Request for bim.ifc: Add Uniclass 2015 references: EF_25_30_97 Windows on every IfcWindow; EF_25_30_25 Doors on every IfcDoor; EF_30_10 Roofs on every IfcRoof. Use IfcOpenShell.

First a look at what the model holds.

```python
import ifcopenshell

model = ifcopenshell.open("bim.ifc")
print(model.schema)
print("classifications:", [c.Name for c in model.by_type("IfcClassification")])
for ifc_class in ("IfcDoor", "IfcRoof", "IfcStair", "IfcWall", "IfcWindow"):
    print(ifc_class, len(model.by_type(ifc_class)))
```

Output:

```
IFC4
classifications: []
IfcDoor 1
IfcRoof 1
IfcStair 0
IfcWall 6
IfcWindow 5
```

```python
import ifcopenshell
import ifcopenshell.api.classification

model = ifcopenshell.open("bim.ifc")

system = ifcopenshell.api.classification.add_classification(model, classification="Uniclass 2015")

codes = {
    "IfcWindow": ("EF_25_30_97", "Windows"),
    "IfcDoor": ("EF_25_30_25", "Doors"),
    "IfcRoof": ("EF_30_10", "Roofs"),
}
for ifc_class, (code, name) in codes.items():
    products = model.by_type(ifc_class)
    ifcopenshell.api.classification.add_reference(
        model, products=products, classification=system, identification=code, name=name
    )
    print(code, len(products))

model.write("bim_v2.ifc")
```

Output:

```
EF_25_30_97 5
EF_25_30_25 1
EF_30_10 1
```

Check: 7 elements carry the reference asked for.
